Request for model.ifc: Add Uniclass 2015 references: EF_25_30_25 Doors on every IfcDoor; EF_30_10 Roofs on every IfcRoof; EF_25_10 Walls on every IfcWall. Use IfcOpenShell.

First a look at what the model holds.

```python
import ifcopenshell

model = ifcopenshell.open("model.ifc")
print(model.schema)
print("classifications:", [c.Name for c in model.by_type("IfcClassification")])
for ifc_class in ("IfcDoor", "IfcRoof", "IfcStair", "IfcWall", "IfcWindow"):
    print(ifc_class, len(model.by_type(ifc_class)))
```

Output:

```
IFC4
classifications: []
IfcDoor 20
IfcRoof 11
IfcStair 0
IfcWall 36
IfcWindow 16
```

```python
import ifcopenshell
import ifcopenshell.api.classification

model = ifcopenshell.open("model.ifc")

system = ifcopenshell.api.classification.add_classification(model, classification="Uniclass 2015")

codes = {
    "IfcDoor": ("EF_25_30_25", "Doors"),
    "IfcRoof": ("EF_30_10", "Roofs"),
    "IfcWall": ("EF_25_10", "Walls"),
}
for ifc_class, (code, name) in codes.items():
    products = model.by_type(ifc_class)
    ifcopenshell.api.classification.add_reference(
        model, products=products, classification=system, identification=code, name=name
    )
    print(code, len(products))

model.write("model_updated.ifc")
```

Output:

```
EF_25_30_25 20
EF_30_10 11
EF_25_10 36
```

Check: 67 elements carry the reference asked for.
